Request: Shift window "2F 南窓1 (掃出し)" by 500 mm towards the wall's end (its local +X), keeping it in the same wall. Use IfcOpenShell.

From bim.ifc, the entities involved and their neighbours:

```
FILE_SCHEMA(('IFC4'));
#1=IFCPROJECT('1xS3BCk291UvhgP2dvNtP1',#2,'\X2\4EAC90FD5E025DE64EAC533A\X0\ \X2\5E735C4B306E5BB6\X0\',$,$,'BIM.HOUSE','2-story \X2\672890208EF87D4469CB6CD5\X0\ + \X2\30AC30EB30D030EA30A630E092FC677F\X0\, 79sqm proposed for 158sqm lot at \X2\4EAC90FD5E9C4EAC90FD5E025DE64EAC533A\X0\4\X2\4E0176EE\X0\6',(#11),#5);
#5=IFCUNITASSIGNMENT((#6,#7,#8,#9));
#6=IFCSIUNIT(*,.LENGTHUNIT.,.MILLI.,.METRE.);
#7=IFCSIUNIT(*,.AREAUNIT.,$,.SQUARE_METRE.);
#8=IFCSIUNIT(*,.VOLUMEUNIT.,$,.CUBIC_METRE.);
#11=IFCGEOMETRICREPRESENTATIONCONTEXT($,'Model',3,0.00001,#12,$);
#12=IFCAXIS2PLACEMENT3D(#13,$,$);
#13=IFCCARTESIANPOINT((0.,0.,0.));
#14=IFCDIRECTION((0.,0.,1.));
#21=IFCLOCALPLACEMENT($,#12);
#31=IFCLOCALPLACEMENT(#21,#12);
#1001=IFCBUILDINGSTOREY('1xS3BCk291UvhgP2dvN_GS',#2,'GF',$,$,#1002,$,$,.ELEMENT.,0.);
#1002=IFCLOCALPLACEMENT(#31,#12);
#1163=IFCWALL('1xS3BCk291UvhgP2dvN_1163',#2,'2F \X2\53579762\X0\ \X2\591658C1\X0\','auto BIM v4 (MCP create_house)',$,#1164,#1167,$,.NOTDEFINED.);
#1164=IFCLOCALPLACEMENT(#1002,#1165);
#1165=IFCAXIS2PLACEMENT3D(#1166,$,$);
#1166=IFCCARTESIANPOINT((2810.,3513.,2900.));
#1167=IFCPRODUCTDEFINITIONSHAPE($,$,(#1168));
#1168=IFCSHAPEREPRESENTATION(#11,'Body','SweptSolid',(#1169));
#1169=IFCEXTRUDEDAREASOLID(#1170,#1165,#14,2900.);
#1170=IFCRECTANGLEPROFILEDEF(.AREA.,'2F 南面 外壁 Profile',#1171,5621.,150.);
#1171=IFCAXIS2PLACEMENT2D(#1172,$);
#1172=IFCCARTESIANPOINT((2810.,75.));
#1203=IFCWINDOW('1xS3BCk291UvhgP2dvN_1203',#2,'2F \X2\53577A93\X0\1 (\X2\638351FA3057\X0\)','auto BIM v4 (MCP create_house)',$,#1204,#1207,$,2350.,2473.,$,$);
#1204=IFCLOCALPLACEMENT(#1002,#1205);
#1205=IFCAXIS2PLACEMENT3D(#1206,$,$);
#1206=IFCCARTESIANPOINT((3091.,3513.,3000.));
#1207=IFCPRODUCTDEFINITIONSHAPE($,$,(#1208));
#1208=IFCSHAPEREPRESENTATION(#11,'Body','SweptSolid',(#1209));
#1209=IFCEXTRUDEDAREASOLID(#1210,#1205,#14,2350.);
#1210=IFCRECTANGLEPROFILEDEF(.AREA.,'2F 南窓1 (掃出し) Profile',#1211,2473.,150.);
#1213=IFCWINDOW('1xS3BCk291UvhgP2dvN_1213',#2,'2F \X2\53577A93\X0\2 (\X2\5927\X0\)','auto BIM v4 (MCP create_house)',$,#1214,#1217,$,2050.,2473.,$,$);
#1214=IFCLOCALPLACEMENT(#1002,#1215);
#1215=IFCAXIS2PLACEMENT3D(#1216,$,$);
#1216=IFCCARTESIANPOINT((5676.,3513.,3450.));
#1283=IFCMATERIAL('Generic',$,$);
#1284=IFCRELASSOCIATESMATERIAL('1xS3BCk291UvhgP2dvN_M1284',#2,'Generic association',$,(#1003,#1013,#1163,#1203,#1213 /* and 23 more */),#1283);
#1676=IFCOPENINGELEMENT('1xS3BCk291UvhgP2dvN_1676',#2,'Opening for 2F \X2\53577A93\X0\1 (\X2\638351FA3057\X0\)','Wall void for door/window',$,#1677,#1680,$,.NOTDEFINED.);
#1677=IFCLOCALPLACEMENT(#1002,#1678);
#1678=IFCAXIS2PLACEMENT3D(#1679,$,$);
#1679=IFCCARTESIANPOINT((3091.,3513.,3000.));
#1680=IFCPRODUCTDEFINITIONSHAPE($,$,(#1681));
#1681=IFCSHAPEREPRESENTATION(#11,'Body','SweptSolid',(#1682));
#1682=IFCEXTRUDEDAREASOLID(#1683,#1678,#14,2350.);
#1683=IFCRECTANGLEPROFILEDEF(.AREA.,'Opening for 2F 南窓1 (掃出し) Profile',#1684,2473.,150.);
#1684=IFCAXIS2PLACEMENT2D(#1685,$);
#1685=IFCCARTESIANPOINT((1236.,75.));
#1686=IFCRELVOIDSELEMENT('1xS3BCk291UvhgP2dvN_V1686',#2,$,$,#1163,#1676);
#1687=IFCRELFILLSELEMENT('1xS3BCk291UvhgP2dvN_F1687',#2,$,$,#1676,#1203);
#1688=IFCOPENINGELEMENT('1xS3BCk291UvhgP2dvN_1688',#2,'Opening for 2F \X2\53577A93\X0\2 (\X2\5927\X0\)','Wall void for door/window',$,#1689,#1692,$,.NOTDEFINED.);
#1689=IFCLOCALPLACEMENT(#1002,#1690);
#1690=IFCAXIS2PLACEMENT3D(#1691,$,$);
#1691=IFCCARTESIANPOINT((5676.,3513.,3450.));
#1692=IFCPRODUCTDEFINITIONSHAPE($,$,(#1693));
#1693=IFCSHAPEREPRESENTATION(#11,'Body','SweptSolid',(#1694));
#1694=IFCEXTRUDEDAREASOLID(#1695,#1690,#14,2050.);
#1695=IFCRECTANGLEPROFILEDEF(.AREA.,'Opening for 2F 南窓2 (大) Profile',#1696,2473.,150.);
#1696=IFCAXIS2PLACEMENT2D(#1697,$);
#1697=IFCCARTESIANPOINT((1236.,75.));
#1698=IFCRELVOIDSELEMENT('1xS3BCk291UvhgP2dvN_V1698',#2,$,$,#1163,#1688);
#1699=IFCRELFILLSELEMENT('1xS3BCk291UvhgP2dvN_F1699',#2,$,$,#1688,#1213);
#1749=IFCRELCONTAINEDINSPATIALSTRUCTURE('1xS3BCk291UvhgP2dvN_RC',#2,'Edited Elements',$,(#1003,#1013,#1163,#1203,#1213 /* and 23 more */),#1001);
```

```python
import ifcopenshell
import ifcopenshell.api.geometry
import ifcopenshell.util.placement

model = ifcopenshell.open("bim.ifc")

window = model.by_guid("1xS3BCk291UvhgP2dvN_1203")
opening = window.FillsVoids[0].RelatingOpeningElement
wall = opening.VoidsElements[0].RelatingBuildingElement

wall_matrix = ifcopenshell.util.placement.get_local_placement(wall.ObjectPlacement)
shift = wall_matrix[:3, 0] * 500.0
before = ifcopenshell.util.placement.get_local_placement(window.ObjectPlacement)[:3, 3].copy()

# The window is not placed relative to its opening, so move both.
for product in (opening, window):
    matrix = ifcopenshell.util.placement.get_local_placement(product.ObjectPlacement)
    matrix[:3, 3] += shift
    ifcopenshell.api.geometry.edit_object_placement(model, product=product, matrix=matrix, is_si=False)

after = ifcopenshell.util.placement.get_local_placement(window.ObjectPlacement)[:3, 3]
print("window moved by", (after - before).round(3) + 0.0)

model.write("bim-out.ifc")
```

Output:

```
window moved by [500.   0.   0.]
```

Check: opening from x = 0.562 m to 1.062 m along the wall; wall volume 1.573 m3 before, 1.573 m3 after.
